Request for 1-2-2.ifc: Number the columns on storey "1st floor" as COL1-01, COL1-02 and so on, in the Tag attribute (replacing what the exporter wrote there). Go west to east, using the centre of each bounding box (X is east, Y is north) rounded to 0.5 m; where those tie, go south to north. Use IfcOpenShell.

First a look at what the model holds.

```python
import ifcopenshell
import ifcopenshell.util.element
import ifcopenshell.util.placement

model = ifcopenshell.open("1-2-2.ifc")
print(model.schema)
storey = next(s for s in model.by_type("IfcBuildingStorey") if s.Name == "1st floor")
columns = [e for e in ifcopenshell.util.element.get_decomposition(storey) if e.is_a("IfcColumn")]
for e in sorted(columns, key=lambda e: e.id()):
    origin = ifcopenshell.util.placement.get_local_placement(e.ObjectPlacement)[:3, 3]
    print(e.id(), e.Tag, e.Name, origin.round(2) + 0.0, sep=" | ")
```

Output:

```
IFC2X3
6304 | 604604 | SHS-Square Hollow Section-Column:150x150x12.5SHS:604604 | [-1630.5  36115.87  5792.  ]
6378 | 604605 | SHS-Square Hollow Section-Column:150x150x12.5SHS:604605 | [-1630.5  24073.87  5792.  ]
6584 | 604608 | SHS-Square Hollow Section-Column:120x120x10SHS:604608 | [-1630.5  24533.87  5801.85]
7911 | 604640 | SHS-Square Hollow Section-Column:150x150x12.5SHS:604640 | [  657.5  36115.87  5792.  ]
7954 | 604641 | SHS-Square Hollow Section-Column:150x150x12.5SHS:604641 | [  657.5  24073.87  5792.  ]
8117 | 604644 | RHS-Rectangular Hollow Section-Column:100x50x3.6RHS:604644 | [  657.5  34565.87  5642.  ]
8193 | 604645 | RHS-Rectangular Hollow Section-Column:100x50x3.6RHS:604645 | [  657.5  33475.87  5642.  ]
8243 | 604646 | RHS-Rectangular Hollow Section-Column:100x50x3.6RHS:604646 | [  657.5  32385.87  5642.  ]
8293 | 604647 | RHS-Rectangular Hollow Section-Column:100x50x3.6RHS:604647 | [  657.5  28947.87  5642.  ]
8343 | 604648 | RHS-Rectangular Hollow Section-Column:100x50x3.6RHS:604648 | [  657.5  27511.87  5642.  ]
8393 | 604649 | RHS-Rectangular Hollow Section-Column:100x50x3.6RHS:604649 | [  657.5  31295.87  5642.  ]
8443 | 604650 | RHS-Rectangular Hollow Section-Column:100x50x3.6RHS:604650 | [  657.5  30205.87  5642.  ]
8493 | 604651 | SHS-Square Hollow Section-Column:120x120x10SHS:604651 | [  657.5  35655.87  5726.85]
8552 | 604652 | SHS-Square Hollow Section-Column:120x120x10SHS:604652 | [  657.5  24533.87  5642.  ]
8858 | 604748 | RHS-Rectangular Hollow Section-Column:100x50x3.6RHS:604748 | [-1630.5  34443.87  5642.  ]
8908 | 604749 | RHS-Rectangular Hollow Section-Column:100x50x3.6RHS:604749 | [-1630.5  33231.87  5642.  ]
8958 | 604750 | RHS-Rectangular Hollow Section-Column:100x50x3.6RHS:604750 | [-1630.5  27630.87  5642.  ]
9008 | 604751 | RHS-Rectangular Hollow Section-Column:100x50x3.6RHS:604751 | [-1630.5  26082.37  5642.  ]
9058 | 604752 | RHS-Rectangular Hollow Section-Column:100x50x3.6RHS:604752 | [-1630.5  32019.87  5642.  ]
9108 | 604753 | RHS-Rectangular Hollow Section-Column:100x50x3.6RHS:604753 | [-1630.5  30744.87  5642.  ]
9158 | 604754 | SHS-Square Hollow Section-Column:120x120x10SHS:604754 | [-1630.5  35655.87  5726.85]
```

```python
import ifcopenshell
import ifcopenshell.geom
import ifcopenshell.util.element
import ifcopenshell.util.shape

model = ifcopenshell.open("1-2-2.ifc")
settings = ifcopenshell.geom.settings()
settings.set("use-world-coords", True)


def centre(element):
    shape = ifcopenshell.geom.create_shape(settings, element)
    return ifcopenshell.util.shape.get_bbox_centroid(shape.geometry)


storey = next(s for s in model.by_type("IfcBuildingStorey") if s.Name == "1st floor")
columns = [e for e in ifcopenshell.util.element.get_decomposition(storey) if e.is_a("IfcColumn")]

# Insertion points can sit at a corner or the storey origin, so sort by the geometry (in metres).
centres = {e: centre(e) for e in columns}
columns.sort(key=lambda e: (round(centres[e][0] / 0.5), centres[e][1]))

for i, e in enumerate(columns, start=1):
    number = f"COL1-{i:02d}"
    e.Tag = number
    print(e.id(), number)

model.write("1-2-2_updated.ifc")
```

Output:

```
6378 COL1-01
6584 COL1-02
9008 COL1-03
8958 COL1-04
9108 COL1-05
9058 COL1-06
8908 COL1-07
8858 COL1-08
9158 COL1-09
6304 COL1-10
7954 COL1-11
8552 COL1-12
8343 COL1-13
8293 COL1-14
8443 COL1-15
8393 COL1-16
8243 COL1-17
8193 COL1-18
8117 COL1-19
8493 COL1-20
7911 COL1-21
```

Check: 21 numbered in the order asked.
